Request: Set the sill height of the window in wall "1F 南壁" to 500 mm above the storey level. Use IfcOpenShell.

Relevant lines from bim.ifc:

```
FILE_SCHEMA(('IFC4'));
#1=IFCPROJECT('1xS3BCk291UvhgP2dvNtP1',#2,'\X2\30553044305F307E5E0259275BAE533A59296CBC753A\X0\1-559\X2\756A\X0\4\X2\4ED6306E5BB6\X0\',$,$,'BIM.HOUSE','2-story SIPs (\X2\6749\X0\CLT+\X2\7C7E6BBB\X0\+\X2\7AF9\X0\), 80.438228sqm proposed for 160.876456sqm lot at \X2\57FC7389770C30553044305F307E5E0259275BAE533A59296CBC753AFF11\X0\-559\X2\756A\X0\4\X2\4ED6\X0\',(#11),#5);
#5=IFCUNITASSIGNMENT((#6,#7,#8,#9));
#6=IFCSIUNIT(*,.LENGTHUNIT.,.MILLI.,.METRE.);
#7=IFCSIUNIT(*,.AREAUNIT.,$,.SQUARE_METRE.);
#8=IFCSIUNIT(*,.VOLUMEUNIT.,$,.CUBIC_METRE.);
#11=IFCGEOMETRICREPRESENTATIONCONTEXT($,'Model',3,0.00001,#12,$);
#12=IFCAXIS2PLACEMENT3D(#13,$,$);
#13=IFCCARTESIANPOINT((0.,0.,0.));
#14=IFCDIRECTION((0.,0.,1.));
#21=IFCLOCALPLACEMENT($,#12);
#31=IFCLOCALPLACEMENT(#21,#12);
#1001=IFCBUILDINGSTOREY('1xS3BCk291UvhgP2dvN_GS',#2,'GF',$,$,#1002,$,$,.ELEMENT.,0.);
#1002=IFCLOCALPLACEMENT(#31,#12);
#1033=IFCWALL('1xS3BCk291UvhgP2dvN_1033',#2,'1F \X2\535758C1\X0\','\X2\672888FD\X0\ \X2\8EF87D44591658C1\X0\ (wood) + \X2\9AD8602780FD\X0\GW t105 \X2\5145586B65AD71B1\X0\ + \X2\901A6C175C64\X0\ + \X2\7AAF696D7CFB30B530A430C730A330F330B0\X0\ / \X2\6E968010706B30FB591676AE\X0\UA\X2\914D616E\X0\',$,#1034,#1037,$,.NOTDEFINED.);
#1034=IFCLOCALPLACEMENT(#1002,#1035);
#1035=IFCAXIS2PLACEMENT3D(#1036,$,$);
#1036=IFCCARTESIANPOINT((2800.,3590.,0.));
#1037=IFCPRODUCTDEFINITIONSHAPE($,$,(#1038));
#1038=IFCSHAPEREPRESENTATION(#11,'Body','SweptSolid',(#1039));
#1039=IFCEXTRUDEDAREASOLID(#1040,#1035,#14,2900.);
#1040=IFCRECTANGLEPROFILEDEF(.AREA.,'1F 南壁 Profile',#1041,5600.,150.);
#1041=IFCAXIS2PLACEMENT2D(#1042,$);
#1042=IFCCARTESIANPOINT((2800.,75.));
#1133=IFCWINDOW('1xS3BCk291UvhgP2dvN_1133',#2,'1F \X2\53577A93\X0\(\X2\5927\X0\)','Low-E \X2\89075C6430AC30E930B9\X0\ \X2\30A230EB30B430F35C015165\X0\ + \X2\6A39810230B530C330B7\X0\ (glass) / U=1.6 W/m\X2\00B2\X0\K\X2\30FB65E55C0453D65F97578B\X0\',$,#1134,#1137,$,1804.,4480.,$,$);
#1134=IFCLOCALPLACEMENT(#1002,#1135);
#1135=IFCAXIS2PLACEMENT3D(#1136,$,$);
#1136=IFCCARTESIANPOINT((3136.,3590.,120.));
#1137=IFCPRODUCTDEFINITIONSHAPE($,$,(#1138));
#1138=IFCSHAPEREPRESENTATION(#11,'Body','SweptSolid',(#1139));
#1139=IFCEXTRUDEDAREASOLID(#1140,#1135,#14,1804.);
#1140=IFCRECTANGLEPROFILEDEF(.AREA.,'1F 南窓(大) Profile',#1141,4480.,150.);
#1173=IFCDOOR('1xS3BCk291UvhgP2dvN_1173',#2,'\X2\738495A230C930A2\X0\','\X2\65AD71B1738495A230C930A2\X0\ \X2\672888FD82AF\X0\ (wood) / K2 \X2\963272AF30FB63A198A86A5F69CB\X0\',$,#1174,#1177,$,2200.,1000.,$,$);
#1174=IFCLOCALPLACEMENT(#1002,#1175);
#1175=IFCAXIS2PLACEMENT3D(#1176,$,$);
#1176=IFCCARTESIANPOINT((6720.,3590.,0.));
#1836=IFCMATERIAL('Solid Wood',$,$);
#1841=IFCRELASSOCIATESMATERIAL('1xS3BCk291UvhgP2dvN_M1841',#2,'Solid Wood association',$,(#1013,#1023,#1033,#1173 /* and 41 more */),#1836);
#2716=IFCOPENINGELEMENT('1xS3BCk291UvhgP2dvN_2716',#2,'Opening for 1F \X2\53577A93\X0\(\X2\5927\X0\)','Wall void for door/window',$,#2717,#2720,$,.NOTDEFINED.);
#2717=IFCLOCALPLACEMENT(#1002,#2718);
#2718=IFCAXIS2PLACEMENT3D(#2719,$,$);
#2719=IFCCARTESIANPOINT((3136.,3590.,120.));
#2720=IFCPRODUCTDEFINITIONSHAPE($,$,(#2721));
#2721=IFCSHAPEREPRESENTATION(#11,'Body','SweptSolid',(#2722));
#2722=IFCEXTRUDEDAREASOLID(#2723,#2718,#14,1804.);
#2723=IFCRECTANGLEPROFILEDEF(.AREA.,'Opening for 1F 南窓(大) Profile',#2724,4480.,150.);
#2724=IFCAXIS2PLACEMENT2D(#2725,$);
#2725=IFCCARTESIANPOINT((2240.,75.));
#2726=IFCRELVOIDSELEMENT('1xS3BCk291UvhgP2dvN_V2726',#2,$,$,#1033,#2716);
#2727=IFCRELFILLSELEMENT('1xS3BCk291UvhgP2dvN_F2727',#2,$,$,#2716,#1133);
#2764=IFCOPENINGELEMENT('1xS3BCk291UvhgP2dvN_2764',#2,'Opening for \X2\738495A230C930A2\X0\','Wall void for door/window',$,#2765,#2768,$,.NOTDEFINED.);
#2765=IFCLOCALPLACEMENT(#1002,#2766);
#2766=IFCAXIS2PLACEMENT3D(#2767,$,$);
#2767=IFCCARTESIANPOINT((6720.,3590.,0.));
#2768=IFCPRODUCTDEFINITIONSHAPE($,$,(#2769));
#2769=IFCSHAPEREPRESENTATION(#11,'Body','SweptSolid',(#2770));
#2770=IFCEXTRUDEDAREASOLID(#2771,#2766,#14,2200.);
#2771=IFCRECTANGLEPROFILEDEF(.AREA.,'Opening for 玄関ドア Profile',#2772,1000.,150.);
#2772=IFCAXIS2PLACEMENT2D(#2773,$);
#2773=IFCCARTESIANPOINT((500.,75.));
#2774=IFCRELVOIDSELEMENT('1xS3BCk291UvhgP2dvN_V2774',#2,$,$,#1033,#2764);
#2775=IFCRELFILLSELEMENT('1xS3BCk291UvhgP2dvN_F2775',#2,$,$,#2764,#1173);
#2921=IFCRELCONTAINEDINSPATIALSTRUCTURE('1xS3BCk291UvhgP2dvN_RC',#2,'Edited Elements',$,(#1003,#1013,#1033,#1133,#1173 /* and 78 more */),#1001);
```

```python
import numpy as np
import ifcopenshell
import ifcopenshell.api.geometry
import ifcopenshell.geom
import ifcopenshell.util.element
import ifcopenshell.util.placement
import ifcopenshell.util.shape
import ifcopenshell.util.unit

model = ifcopenshell.open("bim.ifc")
unit_scale = ifcopenshell.util.unit.calculate_unit_scale(model)

window = model.by_guid("1xS3BCk291UvhgP2dvN_1133")
opening = window.FillsVoids[0].RelatingOpeningElement
storey = ifcopenshell.util.element.get_container(window, ifc_class="IfcBuildingStorey")
level = ifcopenshell.util.placement.get_local_placement(storey.ObjectPlacement)[2, 3]

# The opening's origin need not be at the sill, so measure its lowest point.
shape = ifcopenshell.geom.create_shape(ifcopenshell.geom.settings(), opening)
bottom = ifcopenshell.util.shape.get_shape_bottom_elevation(shape, shape.geometry) / unit_scale
dz = level + 0.5 / unit_scale - bottom

shift = np.array([0.0, 0.0, dz])
# The window is not placed relative to its opening, so move both.
for product in (opening, window):
    matrix = ifcopenshell.util.placement.get_local_placement(product.ObjectPlacement)
    matrix[:3, 3] += shift
    ifcopenshell.api.geometry.edit_object_placement(model, product=product, matrix=matrix, is_si=False)

print(f"moved by {dz * unit_scale:+.3f} m")

model.write("bim_v2.ifc")
```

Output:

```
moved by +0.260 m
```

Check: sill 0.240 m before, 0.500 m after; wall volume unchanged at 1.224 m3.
